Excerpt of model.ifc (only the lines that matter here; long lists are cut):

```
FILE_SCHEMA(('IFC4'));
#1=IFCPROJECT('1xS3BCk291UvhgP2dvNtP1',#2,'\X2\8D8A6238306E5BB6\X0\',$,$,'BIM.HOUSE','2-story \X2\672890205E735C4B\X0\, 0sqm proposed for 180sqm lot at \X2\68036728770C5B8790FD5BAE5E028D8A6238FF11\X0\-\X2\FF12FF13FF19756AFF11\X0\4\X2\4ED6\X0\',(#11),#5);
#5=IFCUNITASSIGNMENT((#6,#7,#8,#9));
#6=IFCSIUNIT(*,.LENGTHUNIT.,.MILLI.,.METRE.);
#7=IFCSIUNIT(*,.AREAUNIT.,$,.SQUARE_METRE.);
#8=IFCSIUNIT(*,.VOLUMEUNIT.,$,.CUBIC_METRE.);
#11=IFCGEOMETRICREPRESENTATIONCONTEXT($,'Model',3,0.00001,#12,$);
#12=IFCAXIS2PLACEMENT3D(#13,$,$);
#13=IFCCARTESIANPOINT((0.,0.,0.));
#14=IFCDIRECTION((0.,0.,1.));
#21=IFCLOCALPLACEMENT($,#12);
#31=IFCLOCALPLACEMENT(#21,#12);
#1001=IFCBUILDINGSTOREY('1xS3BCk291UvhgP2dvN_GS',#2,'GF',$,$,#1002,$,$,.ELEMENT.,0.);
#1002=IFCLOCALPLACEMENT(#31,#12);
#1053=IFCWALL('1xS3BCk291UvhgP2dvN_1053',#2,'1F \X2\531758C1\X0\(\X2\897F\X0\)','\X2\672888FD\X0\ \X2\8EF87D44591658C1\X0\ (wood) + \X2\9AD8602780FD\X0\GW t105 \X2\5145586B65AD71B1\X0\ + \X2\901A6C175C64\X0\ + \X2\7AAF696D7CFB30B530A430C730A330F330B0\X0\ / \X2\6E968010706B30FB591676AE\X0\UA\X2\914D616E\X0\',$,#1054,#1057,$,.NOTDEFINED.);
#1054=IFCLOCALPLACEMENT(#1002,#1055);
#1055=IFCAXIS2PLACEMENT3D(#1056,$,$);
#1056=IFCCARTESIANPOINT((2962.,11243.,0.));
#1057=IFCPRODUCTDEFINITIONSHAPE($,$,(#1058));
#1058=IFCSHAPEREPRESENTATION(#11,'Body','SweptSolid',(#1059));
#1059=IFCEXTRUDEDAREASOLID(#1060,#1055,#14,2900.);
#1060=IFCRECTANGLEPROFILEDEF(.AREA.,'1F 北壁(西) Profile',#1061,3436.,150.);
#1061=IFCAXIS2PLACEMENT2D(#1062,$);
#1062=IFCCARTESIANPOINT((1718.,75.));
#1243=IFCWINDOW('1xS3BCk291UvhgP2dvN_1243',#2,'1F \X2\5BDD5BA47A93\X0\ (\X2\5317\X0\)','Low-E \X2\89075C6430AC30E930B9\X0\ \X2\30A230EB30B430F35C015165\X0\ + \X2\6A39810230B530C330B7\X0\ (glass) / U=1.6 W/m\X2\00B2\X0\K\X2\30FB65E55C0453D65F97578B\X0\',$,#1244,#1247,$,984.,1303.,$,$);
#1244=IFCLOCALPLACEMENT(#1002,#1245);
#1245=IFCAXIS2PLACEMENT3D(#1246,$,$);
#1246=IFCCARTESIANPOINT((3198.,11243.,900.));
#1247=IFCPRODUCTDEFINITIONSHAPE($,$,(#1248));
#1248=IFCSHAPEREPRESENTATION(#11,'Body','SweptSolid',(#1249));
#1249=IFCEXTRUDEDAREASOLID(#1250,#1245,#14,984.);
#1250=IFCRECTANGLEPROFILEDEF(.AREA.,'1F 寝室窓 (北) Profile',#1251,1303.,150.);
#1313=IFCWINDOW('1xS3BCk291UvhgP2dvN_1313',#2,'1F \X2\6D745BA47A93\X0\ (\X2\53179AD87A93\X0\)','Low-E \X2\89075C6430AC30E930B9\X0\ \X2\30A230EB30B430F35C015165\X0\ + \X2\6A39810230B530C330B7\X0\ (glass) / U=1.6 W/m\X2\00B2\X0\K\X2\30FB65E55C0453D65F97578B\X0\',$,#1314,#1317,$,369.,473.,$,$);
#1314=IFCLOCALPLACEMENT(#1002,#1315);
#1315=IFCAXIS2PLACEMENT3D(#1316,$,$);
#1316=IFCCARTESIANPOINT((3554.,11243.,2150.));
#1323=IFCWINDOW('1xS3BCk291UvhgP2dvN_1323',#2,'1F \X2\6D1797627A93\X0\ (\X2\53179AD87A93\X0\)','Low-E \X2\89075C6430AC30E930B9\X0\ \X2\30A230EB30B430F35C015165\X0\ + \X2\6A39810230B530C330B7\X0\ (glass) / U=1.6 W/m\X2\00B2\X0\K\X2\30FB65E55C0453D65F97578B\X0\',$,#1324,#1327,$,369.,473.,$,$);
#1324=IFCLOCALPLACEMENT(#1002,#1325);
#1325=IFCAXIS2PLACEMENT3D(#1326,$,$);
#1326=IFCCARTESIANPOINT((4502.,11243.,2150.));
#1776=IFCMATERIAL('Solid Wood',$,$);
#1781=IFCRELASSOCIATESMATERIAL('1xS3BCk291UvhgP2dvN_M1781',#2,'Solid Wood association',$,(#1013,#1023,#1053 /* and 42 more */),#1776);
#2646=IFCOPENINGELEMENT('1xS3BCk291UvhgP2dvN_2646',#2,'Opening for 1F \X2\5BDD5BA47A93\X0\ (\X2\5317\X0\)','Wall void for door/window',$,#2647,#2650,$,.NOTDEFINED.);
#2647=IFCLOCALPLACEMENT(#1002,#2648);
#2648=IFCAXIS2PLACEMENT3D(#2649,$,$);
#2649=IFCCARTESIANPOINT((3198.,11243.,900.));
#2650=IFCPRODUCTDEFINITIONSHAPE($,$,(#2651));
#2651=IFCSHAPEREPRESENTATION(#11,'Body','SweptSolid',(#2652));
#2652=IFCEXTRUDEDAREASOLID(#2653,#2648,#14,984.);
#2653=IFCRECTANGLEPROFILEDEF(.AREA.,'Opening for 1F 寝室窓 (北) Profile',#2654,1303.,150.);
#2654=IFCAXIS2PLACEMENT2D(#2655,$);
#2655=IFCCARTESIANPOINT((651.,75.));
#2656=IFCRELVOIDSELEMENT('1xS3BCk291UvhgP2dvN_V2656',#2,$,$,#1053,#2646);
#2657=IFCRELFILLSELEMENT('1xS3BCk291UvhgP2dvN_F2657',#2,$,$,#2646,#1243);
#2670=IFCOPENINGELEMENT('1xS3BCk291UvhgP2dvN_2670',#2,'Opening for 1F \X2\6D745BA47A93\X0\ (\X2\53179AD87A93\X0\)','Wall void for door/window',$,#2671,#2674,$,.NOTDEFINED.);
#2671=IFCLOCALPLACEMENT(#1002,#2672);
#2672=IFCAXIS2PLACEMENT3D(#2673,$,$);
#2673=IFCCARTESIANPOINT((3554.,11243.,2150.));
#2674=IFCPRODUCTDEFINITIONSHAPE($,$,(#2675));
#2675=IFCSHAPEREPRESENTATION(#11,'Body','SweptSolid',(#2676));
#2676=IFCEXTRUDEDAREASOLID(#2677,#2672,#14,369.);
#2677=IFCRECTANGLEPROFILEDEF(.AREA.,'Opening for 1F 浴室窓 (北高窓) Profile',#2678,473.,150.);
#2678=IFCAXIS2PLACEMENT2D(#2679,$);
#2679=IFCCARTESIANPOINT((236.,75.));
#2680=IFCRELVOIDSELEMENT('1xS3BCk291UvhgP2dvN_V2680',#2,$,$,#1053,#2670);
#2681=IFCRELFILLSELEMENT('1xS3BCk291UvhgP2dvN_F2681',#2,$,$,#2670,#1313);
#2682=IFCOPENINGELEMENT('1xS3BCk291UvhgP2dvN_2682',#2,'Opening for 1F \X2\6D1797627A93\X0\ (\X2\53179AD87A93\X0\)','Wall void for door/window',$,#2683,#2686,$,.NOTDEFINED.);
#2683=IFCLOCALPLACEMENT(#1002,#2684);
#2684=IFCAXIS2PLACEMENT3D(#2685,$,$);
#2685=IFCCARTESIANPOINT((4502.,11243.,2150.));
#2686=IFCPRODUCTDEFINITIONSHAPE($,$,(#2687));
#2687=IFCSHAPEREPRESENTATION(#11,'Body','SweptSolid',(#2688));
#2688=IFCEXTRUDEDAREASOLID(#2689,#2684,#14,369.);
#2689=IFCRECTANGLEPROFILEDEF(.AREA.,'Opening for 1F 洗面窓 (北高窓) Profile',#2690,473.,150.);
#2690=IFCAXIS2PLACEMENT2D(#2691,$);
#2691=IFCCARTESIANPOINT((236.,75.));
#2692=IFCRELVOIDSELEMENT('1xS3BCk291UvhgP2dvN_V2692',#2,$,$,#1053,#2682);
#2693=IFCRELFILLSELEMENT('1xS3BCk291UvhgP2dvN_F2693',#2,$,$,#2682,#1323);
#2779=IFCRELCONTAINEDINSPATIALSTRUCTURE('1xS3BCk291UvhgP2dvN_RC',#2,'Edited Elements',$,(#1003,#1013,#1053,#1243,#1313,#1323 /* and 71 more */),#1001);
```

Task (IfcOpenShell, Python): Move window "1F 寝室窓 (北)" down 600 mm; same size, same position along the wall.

```python
import numpy as np
import ifcopenshell
import ifcopenshell.api.geometry
import ifcopenshell.util.placement
import ifcopenshell.util.unit

model = ifcopenshell.open("model.ifc")
unit_scale = ifcopenshell.util.unit.calculate_unit_scale(model)

window = model.by_id(1243)
opening = window.FillsVoids[0].RelatingOpeningElement
dz = -600.0

shift = np.array([0.0, 0.0, dz])
# The window is not placed relative to its opening, so move both.
for product in (opening, window):
    matrix = ifcopenshell.util.placement.get_local_placement(product.ObjectPlacement)
    matrix[:3, 3] += shift
    ifcopenshell.api.geometry.edit_object_placement(model, product=product, matrix=matrix, is_si=False)

print(f"moved by {dz * unit_scale:+.3f} m")

model.write("model_edited.ifc")
```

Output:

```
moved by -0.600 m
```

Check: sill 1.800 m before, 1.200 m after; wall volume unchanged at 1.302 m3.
